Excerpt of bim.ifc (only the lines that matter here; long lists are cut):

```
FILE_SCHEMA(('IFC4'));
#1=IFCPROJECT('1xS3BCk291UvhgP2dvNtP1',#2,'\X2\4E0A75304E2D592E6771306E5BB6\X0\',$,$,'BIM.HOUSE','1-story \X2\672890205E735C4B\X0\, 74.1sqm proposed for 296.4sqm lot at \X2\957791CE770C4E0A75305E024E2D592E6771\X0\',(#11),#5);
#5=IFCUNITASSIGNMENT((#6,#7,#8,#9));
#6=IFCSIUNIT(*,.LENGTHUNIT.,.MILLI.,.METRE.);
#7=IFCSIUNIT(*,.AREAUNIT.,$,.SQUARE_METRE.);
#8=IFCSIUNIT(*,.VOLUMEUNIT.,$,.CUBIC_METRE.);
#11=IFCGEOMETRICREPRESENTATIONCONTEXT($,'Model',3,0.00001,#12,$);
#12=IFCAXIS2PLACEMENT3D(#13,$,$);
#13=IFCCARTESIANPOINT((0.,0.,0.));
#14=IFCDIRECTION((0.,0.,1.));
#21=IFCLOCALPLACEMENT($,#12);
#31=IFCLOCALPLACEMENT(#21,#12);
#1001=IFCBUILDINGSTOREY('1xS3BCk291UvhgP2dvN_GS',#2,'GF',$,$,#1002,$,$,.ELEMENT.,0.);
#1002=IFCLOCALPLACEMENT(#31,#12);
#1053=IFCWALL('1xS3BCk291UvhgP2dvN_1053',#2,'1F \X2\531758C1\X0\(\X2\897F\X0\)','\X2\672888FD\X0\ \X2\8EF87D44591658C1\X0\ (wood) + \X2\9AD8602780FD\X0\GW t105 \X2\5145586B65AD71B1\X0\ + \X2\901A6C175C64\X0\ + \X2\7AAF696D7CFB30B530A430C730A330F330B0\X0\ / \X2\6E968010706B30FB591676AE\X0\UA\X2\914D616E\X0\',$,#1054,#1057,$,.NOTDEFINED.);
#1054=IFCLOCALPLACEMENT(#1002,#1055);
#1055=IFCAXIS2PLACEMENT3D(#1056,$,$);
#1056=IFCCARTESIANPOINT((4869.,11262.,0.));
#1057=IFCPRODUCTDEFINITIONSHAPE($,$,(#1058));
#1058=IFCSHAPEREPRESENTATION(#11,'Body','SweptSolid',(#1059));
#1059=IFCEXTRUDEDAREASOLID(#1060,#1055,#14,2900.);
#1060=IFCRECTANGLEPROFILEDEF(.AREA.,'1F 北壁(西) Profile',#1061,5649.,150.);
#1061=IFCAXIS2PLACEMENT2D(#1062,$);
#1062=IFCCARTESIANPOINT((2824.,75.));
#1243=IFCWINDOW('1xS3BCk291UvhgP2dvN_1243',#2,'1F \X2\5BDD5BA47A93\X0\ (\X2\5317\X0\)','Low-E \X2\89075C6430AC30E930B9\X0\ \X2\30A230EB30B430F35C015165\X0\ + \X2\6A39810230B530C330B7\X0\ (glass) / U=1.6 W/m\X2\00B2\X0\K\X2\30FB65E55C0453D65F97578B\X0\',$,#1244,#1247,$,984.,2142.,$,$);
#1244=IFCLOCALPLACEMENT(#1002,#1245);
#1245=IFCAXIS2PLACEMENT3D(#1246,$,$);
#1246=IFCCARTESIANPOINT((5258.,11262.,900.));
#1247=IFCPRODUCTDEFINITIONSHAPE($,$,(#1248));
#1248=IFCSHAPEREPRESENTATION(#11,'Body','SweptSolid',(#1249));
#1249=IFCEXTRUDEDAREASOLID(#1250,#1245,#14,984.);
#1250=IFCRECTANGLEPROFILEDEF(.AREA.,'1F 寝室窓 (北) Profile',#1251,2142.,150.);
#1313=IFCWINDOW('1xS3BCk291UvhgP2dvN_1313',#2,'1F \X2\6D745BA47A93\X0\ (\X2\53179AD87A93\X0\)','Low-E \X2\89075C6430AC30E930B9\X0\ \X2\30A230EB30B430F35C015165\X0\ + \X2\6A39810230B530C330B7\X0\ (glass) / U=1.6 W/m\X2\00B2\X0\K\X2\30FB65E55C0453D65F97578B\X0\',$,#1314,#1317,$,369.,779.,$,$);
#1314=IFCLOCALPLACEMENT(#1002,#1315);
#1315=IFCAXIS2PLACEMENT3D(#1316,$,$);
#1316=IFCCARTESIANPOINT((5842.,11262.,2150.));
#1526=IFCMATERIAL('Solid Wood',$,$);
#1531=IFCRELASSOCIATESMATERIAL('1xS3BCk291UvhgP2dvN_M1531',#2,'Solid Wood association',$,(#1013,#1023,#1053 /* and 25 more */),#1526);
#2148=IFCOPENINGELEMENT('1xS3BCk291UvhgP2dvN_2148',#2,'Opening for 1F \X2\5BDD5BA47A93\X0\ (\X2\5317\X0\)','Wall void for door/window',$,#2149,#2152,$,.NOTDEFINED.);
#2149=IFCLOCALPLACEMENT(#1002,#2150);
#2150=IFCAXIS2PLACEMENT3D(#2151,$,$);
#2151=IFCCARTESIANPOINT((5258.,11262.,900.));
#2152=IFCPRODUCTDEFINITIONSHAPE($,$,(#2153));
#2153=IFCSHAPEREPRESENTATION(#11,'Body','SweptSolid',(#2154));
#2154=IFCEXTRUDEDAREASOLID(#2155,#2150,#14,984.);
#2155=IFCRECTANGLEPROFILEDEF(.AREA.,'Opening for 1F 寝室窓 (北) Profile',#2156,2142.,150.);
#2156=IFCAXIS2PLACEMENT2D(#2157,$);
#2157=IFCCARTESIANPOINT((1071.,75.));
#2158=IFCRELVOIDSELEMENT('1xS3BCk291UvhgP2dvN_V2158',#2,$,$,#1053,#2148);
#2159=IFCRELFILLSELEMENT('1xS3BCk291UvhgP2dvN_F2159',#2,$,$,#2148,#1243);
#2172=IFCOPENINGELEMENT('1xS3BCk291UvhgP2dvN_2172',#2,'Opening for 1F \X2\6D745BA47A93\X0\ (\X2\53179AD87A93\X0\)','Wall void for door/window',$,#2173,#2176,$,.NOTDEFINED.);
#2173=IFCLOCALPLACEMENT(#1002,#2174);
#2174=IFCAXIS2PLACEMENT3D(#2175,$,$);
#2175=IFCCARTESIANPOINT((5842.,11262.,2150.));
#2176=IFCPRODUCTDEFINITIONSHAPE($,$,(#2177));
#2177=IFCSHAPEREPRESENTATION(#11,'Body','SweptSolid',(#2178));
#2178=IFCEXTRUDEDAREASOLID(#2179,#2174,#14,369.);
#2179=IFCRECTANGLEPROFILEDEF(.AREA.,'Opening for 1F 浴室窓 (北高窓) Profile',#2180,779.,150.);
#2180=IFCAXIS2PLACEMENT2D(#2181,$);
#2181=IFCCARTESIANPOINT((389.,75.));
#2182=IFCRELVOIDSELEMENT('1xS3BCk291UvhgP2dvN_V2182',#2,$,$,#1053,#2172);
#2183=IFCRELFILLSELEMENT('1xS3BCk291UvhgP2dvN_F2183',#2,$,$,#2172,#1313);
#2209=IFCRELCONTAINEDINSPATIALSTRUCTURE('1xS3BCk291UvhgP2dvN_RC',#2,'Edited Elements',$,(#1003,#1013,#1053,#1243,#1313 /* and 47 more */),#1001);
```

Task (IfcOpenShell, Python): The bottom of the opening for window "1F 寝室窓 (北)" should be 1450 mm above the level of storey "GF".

```python
import numpy as np
import ifcopenshell
import ifcopenshell.api.geometry
import ifcopenshell.geom
import ifcopenshell.util.element
import ifcopenshell.util.placement
import ifcopenshell.util.shape
import ifcopenshell.util.unit

model = ifcopenshell.open("bim.ifc")
unit_scale = ifcopenshell.util.unit.calculate_unit_scale(model)

window = model.by_guid("1xS3BCk291UvhgP2dvN_1243")
opening = window.FillsVoids[0].RelatingOpeningElement
storey = ifcopenshell.util.element.get_container(window, ifc_class="IfcBuildingStorey")
level = ifcopenshell.util.placement.get_local_placement(storey.ObjectPlacement)[2, 3]

# The opening's origin need not be at the sill, so measure its lowest point.
shape = ifcopenshell.geom.create_shape(ifcopenshell.geom.settings(), opening)
bottom = ifcopenshell.util.shape.get_shape_bottom_elevation(shape, shape.geometry) / unit_scale
dz = level + 1.45 / unit_scale - bottom

shift = np.array([0.0, 0.0, dz])
# The window is not placed relative to its opening, so move both.
for product in (opening, window):
    matrix = ifcopenshell.util.placement.get_local_placement(product.ObjectPlacement)
    matrix[:3, 3] += shift
    ifcopenshell.api.geometry.edit_object_placement(model, product=product, matrix=matrix, is_si=False)

print(f"moved by {dz * unit_scale:+.3f} m")

model.write("bim_edited.ifc")
```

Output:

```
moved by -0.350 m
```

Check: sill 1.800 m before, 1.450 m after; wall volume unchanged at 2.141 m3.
